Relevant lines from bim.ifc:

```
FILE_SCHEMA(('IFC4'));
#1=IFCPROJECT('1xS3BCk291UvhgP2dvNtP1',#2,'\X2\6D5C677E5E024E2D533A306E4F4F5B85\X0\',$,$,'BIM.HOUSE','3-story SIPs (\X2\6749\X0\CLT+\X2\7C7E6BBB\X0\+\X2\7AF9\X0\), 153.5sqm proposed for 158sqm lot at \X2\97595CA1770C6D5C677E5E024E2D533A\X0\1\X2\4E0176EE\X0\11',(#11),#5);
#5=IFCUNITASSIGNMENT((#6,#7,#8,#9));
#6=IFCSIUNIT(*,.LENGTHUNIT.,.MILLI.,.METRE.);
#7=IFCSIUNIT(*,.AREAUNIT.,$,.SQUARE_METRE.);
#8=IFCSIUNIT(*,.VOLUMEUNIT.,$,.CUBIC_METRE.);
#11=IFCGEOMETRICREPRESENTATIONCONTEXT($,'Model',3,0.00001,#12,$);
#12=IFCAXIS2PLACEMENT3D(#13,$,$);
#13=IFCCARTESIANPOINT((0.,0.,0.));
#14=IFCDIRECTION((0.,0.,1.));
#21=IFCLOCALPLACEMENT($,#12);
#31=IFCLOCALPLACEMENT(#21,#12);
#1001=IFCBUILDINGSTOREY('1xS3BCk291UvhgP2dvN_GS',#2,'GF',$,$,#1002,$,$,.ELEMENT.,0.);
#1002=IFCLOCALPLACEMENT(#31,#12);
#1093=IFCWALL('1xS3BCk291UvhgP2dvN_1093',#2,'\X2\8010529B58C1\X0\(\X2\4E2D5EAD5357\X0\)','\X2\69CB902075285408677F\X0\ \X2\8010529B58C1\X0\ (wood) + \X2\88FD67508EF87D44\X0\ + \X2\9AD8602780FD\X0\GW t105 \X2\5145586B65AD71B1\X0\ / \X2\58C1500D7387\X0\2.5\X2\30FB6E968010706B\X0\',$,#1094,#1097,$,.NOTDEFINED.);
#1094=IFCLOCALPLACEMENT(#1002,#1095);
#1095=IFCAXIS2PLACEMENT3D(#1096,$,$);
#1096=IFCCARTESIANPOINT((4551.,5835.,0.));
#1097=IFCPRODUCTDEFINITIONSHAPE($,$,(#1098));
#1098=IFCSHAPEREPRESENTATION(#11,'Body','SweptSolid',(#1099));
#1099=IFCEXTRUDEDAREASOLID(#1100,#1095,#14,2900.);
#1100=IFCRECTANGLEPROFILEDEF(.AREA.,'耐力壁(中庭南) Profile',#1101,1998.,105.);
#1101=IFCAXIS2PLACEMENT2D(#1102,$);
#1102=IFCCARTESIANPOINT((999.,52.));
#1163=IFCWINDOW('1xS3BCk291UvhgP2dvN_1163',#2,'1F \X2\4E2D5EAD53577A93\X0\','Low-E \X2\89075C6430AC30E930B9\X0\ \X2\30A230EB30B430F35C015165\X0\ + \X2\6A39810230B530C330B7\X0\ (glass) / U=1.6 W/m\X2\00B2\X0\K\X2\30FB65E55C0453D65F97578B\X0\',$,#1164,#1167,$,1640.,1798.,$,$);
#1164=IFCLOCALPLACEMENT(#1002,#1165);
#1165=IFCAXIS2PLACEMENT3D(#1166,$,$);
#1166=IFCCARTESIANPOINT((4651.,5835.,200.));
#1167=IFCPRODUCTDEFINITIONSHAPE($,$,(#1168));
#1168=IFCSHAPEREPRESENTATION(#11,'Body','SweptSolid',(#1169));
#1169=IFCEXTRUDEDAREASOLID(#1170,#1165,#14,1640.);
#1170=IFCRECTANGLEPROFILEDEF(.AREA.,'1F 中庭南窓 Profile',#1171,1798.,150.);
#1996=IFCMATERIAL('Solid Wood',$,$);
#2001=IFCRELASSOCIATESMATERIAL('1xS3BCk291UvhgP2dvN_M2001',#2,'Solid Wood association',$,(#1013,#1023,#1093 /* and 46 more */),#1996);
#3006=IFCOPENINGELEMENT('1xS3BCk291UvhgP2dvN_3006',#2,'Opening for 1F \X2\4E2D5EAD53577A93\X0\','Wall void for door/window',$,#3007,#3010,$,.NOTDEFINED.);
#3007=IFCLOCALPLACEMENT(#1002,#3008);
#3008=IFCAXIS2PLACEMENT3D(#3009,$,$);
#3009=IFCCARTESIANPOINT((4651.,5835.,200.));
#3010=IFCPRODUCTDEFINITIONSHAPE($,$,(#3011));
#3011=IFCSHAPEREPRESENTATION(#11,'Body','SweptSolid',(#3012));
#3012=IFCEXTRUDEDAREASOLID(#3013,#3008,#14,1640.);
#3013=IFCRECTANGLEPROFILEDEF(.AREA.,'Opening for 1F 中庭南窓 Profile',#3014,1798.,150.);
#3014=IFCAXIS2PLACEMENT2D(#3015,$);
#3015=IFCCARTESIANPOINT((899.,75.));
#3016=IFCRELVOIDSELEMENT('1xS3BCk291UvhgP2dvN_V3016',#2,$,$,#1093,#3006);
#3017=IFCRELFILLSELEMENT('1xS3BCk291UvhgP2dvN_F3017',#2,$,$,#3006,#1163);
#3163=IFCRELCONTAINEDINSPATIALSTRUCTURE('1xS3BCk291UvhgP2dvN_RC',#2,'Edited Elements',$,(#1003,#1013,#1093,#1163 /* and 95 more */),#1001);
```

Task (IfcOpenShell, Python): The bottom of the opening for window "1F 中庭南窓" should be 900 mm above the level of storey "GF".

```python
import numpy as np
import ifcopenshell
import ifcopenshell.api.geometry
import ifcopenshell.geom
import ifcopenshell.util.element
import ifcopenshell.util.placement
import ifcopenshell.util.shape
import ifcopenshell.util.unit

model = ifcopenshell.open("bim.ifc")
unit_scale = ifcopenshell.util.unit.calculate_unit_scale(model)

window = model.by_guid("1xS3BCk291UvhgP2dvN_1163")
opening = window.FillsVoids[0].RelatingOpeningElement
storey = ifcopenshell.util.element.get_container(window, ifc_class="IfcBuildingStorey")
level = ifcopenshell.util.placement.get_local_placement(storey.ObjectPlacement)[2, 3]

# The opening's origin need not be at the sill, so measure its lowest point.
shape = ifcopenshell.geom.create_shape(ifcopenshell.geom.settings(), opening)
bottom = ifcopenshell.util.shape.get_shape_bottom_elevation(shape, shape.geometry) / unit_scale
dz = level + 900.0 - bottom

shift = np.array([0.0, 0.0, dz])
# The window is not placed relative to its opening, so move both.
for product in (opening, window):
    matrix = ifcopenshell.util.placement.get_local_placement(product.ObjectPlacement)
    matrix[:3, 3] += shift
    ifcopenshell.api.geometry.edit_object_placement(model, product=product, matrix=matrix, is_si=False)

print(f"moved by {dz * unit_scale:+.3f} m")

model.write("bim-out.ifc")
```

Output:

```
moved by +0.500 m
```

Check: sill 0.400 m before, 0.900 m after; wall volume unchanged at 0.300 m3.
